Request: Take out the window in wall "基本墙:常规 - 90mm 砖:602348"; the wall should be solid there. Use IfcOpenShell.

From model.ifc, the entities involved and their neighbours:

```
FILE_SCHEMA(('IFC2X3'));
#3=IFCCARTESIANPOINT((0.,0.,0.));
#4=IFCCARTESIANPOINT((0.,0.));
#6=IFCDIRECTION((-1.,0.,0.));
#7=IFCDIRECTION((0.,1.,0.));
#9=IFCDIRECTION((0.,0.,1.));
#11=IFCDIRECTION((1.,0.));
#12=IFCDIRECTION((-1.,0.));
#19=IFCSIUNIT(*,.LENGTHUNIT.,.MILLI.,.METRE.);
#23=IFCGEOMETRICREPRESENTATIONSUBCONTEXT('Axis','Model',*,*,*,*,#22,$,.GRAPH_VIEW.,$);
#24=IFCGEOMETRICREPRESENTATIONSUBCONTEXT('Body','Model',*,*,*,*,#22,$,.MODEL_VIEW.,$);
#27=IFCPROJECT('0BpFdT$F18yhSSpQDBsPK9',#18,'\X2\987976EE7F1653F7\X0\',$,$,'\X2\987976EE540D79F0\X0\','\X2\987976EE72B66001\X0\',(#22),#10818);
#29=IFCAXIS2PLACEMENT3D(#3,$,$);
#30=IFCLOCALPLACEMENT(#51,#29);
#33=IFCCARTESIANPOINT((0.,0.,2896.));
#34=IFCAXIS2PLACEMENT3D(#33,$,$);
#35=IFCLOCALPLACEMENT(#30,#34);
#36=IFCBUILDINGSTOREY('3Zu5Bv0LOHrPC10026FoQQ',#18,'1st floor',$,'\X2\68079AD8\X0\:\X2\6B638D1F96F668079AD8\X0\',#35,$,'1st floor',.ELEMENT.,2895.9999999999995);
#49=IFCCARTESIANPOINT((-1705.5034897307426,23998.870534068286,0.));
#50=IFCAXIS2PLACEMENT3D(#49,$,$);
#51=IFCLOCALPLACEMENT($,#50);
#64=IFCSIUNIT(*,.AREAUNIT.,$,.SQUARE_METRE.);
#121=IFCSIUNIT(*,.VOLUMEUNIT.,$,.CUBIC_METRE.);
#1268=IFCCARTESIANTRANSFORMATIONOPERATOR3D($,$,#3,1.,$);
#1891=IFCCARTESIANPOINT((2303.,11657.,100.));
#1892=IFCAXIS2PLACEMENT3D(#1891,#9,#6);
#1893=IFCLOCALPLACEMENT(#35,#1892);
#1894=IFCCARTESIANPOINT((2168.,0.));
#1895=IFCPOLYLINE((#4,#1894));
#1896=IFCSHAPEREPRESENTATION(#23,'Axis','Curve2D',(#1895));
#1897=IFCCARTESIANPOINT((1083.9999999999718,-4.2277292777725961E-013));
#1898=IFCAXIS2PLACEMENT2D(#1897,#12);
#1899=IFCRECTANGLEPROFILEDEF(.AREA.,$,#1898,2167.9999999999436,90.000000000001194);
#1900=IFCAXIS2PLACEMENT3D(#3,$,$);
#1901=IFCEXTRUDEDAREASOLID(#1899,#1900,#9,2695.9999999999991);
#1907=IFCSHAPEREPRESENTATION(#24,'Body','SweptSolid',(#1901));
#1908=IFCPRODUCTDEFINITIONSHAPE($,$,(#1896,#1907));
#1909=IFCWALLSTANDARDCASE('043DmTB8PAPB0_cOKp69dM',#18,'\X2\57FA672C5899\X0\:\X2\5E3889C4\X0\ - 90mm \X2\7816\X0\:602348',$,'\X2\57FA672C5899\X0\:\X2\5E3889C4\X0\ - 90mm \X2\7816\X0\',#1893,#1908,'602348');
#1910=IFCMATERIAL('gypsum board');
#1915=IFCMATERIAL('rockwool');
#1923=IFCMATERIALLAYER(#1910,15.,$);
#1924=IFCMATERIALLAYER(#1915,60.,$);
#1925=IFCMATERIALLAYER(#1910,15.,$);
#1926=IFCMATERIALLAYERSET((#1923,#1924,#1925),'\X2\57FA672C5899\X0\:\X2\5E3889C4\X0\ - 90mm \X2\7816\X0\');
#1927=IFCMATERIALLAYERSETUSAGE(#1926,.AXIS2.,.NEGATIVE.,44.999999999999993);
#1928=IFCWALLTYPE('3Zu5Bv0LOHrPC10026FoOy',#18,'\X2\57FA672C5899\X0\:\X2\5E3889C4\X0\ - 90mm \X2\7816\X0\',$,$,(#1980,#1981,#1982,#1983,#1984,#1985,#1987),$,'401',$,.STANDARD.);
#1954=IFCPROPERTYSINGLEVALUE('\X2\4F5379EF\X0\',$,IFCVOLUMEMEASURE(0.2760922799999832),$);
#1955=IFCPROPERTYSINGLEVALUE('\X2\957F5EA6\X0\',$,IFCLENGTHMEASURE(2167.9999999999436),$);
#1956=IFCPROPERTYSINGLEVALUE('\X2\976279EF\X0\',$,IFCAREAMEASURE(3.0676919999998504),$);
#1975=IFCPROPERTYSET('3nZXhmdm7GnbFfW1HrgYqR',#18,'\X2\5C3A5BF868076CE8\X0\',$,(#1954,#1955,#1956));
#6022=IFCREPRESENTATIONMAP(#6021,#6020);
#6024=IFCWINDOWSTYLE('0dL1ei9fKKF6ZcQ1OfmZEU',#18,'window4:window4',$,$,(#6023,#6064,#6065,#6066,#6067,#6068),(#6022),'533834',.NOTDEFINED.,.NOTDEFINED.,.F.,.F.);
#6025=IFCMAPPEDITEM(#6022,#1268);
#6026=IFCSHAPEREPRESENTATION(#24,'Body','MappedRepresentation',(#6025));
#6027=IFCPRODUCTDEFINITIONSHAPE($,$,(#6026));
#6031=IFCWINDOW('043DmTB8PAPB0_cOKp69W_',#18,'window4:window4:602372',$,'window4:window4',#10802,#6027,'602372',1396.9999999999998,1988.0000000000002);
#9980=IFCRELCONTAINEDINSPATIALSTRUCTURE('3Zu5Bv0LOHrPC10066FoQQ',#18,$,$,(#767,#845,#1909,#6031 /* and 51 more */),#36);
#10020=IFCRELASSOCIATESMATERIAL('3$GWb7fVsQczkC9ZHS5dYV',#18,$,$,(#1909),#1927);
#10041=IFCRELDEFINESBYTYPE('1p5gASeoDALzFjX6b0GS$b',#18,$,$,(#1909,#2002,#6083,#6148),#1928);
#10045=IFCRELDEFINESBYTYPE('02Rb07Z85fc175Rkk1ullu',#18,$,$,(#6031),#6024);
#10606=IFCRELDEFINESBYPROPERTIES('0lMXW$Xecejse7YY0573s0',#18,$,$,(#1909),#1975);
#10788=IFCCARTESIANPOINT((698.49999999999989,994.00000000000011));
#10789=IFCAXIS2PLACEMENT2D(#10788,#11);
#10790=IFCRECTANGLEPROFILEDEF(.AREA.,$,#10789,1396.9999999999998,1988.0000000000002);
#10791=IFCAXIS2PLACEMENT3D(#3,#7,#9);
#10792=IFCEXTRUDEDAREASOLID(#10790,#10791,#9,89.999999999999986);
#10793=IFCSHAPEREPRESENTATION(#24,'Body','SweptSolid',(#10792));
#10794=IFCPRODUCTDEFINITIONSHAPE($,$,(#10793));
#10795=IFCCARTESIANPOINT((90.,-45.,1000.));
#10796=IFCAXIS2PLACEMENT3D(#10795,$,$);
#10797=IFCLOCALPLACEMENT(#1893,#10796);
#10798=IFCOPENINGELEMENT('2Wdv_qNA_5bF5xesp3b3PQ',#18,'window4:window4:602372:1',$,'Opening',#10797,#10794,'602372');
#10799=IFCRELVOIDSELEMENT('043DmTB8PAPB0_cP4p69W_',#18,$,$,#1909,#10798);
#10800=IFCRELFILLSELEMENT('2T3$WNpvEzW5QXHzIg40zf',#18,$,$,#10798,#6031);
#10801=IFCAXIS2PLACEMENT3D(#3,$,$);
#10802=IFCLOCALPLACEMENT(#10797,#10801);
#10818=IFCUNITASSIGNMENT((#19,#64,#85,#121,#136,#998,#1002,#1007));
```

```python
import ifcopenshell
import ifcopenshell.api.feature
import ifcopenshell.api.pset
import ifcopenshell.api.root
import ifcopenshell.geom
import ifcopenshell.util.element
import ifcopenshell.util.shape
import ifcopenshell.util.unit

model = ifcopenshell.open("model.ifc")
area_scale = ifcopenshell.util.unit.calculate_unit_scale(model, "AREAUNIT")
volume_scale = ifcopenshell.util.unit.calculate_unit_scale(model, "VOLUMEUNIT")
settings = ifcopenshell.geom.settings()


def volume(element):
    """Net volume in cubic metres, openings subtracted."""
    shape = ifcopenshell.geom.create_shape(settings, element)
    return ifcopenshell.util.shape.get_volume(shape.geometry)


window = model.by_guid("043DmTB8PAPB0_cOKp69W_")
opening = window.FillsVoids[0].RelatingOpeningElement
wall = opening.VoidsElements[0].RelatingBuildingElement
before = volume(wall)

ifcopenshell.api.root.remove_product(model, product=window)
ifcopenshell.api.feature.remove_feature(model, feature=opening)

after = volume(wall)
thickness = 0.09  # wall thickness in metres

# Update the wall's stored quantities.
pset = model.by_id(ifcopenshell.util.element.get_pset(wall, "尺寸标注", should_inherit=False)["id"])
ifcopenshell.api.pset.edit_pset(model, pset=pset, properties={
    "体积": model.create_entity("IfcVolumeMeasure", after / volume_scale),
    "面积": model.create_entity("IfcAreaMeasure", after / thickness / area_scale),
})

print(f"wall volume {before:.3f} -> {after:.3f} m3")

model.write("model_rev.ifc")
```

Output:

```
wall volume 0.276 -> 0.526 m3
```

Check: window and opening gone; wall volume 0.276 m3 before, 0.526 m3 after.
